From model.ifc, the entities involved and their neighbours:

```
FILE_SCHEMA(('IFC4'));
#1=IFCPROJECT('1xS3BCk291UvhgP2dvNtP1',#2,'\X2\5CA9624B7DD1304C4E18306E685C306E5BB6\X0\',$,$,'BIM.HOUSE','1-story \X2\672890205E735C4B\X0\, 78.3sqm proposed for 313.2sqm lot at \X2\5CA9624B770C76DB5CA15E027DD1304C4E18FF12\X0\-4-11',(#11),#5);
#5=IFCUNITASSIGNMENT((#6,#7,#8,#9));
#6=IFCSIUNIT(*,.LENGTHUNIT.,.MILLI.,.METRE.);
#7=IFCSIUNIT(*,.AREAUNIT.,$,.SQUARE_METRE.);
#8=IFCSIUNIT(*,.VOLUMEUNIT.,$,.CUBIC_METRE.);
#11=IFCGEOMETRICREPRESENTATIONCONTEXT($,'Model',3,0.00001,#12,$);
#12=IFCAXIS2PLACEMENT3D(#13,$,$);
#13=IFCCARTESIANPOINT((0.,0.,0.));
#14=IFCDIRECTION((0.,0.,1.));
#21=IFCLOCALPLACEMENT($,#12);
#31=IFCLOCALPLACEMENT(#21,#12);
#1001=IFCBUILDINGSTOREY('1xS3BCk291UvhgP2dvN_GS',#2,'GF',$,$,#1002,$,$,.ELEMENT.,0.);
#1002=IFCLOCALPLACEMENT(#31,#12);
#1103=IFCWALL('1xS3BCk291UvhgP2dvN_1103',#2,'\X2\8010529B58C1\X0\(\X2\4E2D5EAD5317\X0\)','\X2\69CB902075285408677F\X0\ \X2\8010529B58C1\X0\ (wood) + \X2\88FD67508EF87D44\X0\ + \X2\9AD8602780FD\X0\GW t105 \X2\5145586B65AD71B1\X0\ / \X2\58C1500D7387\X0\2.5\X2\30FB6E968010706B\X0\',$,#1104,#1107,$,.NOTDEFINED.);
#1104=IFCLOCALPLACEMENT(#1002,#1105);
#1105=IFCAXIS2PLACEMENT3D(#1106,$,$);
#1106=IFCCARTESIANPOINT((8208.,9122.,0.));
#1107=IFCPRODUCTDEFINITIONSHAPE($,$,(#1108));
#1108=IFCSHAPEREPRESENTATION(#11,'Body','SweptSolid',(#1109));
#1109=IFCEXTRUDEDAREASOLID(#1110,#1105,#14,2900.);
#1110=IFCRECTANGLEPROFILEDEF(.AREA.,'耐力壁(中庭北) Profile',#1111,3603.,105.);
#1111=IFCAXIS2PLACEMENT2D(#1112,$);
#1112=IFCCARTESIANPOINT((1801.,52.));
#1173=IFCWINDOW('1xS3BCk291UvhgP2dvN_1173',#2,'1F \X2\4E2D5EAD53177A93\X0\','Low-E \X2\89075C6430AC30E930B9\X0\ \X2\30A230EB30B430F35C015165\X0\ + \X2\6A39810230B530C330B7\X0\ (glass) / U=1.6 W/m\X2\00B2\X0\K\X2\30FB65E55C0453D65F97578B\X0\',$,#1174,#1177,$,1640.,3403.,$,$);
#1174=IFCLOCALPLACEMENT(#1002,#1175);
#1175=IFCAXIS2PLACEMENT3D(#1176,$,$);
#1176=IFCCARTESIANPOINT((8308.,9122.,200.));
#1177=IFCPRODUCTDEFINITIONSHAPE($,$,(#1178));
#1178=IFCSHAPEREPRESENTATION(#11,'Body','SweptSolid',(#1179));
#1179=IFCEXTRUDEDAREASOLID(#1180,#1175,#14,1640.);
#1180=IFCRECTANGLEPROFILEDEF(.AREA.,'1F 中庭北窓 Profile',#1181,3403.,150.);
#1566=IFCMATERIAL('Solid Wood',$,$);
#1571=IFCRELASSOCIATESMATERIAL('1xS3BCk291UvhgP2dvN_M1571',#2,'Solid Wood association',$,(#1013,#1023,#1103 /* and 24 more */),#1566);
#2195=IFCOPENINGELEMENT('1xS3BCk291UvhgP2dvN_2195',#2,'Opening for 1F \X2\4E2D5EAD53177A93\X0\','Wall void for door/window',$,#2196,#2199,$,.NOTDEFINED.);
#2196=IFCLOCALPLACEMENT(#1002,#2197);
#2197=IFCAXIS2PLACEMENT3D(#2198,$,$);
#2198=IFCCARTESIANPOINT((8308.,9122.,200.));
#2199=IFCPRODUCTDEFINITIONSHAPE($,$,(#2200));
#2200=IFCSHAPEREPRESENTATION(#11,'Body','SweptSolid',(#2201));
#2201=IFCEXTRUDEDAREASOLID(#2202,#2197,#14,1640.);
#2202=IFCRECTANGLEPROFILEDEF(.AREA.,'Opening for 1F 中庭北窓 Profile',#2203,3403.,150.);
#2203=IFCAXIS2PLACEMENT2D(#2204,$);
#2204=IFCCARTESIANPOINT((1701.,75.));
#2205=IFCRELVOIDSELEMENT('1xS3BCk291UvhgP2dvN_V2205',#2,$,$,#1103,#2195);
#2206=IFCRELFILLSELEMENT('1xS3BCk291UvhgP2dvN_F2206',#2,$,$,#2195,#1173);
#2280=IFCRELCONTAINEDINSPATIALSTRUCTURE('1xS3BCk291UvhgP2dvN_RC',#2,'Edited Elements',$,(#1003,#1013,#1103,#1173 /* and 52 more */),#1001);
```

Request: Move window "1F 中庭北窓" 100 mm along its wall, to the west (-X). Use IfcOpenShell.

```python
import ifcopenshell
import ifcopenshell.api.geometry
import ifcopenshell.util.placement

model = ifcopenshell.open("model.ifc")

window = model.by_id(1173)
opening = window.FillsVoids[0].RelatingOpeningElement
wall = opening.VoidsElements[0].RelatingBuildingElement

wall_matrix = ifcopenshell.util.placement.get_local_placement(wall.ObjectPlacement)
shift = wall_matrix[:3, 0] * -100.0
before = ifcopenshell.util.placement.get_local_placement(window.ObjectPlacement)[:3, 3].copy()

# The window is not placed relative to its opening, so move both.
for product in (opening, window):
    matrix = ifcopenshell.util.placement.get_local_placement(product.ObjectPlacement)
    matrix[:3, 3] += shift
    ifcopenshell.api.geometry.edit_object_placement(model, product=product, matrix=matrix, is_si=False)

after = ifcopenshell.util.placement.get_local_placement(window.ObjectPlacement)[:3, 3]
print("window moved by", (after - before).round(3) + 0.0)

model.write("model_updated.ifc")
```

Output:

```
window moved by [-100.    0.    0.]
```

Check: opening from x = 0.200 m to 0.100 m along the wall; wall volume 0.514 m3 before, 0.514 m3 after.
